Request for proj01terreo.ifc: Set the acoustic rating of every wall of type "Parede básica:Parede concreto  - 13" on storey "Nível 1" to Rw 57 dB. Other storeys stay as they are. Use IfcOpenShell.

First a look at what the model holds.

```python
import ifcopenshell
import ifcopenshell.util.element

model = ifcopenshell.open("proj01terreo.ifc")
print(model.schema)
storey = next(s for s in model.by_type("IfcBuildingStorey") if s.Name == "Nível 1")
walls = [e for e in ifcopenshell.util.element.get_decomposition(storey) if e.is_a("IfcWall")]
seen = {}
for e in walls:
    element_type = ifcopenshell.util.element.get_type(e)
    key = (element_type.Name if element_type != e and element_type else None, ifcopenshell.util.element.get_pset(e, "Pset_WallCommon", "AcousticRating"))
    seen[key] = seen.get(key, 0) + 1
for (name, value), count in sorted(seen.items(), key=str):
    print(count, "x", name, "|", value)
```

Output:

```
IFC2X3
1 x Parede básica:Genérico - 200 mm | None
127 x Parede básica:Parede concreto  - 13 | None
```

```python
import ifcopenshell
import ifcopenshell.api.pset
import ifcopenshell.util.element

model = ifcopenshell.open("proj01terreo.ifc")

storey = next(s for s in model.by_type("IfcBuildingStorey") if s.Name == "Nível 1")
walls = [e for e in ifcopenshell.util.element.get_decomposition(storey) if e.is_a("IfcWall")]

count = 0
for e in walls:
    element_type = ifcopenshell.util.element.get_type(e)
    if element_type in (None, e) or element_type.Name != "Parede básica:Parede concreto  - 13":
        continue
    # add_pset returns the element's existing set when there is one.
    pset = ifcopenshell.api.pset.add_pset(model, product=e, name="Pset_WallCommon")
    ifcopenshell.api.pset.edit_pset(model, pset=pset, properties={"AcousticRating": "Rw 57 dB"})
    count += 1

print(count, "walls updated")

model.write("proj01terreo_rev.ifc")
```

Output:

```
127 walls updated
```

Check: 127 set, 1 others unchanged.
